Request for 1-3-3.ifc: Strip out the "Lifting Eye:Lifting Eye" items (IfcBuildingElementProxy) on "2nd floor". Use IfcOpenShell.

First a look at what the model holds.

```python
import ifcopenshell
import ifcopenshell.util.element

model = ifcopenshell.open("1-3-3.ifc")
print(model.schema)
storey = next(s for s in model.by_type("IfcBuildingStorey") if s.Name == "2nd floor")
proxies = [e for e in ifcopenshell.util.element.get_decomposition(storey) if e.is_a("IfcBuildingElementProxy")]
seen = {}
for e in proxies:
    element_type = ifcopenshell.util.element.get_type(e)
    name = element_type.Name if element_type not in (None, e) else None
    seen[name] = seen.get(name, 0) + 1
for name, count in sorted(seen.items(), key=str):
    print(count, "x", name)
```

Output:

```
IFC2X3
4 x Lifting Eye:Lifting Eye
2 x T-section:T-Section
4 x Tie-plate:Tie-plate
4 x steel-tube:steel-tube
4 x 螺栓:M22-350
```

```python
import ifcopenshell
import ifcopenshell.api.root
import ifcopenshell.util.element

model = ifcopenshell.open("1-3-3.ifc")

storey = next(s for s in model.by_type("IfcBuildingStorey") if s.Name == "2nd floor")
proxies = [e for e in ifcopenshell.util.element.get_decomposition(storey) if e.is_a("IfcBuildingElementProxy")]
targets = [e for e in proxies if (t := ifcopenshell.util.element.get_type(e)) not in (None, e) and t.Name == "Lifting Eye:Lifting Eye"]

for e in targets:
    ifcopenshell.api.root.remove_product(model, product=e)
print(len(targets), "removed")

model.write("1-3-3_edited.ifc")
```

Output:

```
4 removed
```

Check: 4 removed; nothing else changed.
